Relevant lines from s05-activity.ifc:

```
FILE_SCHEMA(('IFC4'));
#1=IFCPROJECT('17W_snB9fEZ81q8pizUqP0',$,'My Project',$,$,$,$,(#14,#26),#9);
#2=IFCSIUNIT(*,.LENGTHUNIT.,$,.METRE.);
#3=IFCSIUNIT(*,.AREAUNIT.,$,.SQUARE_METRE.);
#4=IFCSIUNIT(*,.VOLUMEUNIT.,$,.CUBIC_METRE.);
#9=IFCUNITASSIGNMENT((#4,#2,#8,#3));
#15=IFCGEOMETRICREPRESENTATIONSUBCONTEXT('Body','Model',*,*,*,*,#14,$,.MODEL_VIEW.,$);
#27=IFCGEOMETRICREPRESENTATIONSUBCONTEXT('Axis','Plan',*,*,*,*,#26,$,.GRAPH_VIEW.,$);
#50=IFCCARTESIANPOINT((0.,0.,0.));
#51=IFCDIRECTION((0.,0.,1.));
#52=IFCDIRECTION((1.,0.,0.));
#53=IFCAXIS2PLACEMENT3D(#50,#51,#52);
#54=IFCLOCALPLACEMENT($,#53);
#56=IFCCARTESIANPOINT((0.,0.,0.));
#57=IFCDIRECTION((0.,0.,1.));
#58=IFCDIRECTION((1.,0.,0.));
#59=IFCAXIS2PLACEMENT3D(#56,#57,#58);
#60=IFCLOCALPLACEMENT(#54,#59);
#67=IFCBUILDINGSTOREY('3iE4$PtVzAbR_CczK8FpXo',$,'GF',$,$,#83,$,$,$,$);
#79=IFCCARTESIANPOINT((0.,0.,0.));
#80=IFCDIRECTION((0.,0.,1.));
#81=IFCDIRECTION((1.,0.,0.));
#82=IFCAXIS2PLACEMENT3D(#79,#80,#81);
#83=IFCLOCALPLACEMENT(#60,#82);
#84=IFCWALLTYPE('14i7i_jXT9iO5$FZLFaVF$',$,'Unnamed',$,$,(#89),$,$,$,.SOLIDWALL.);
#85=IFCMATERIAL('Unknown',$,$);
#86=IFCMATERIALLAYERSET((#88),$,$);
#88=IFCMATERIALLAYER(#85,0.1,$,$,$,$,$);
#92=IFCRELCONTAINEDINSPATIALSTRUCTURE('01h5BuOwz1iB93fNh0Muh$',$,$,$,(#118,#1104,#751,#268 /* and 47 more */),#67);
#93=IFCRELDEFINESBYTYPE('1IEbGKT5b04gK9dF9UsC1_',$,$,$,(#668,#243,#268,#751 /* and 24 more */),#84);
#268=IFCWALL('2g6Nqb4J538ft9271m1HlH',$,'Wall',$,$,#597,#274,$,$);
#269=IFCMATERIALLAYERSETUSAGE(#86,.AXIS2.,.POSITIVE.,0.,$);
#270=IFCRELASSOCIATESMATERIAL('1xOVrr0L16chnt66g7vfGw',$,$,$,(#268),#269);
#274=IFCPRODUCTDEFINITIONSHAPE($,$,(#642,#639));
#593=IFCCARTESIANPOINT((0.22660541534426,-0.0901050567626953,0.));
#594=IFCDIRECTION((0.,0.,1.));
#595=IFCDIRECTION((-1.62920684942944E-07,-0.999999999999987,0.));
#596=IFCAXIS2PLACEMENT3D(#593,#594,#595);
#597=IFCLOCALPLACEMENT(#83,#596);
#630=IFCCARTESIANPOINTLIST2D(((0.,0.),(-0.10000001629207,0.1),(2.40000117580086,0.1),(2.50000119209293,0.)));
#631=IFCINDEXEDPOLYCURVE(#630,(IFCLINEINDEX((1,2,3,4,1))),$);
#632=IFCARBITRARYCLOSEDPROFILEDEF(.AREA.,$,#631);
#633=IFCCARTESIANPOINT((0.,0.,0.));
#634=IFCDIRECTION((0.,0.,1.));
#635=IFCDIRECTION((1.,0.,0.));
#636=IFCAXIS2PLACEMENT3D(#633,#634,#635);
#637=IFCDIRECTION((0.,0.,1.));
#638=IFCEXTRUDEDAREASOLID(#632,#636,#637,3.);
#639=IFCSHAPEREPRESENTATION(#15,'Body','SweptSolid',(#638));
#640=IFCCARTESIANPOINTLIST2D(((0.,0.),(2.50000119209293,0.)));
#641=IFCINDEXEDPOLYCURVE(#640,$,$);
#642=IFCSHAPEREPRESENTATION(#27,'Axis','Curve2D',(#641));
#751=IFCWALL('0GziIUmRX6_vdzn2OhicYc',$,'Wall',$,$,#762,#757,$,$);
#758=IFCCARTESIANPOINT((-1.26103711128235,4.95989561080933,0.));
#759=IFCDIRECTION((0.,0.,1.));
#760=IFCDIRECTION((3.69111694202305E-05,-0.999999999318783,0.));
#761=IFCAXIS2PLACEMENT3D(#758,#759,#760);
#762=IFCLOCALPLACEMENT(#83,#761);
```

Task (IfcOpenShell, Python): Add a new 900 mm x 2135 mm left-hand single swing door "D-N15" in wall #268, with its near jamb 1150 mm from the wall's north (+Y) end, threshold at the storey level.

```python
import numpy as np
import ifcopenshell
import ifcopenshell.api.feature
import ifcopenshell.api.geometry
import ifcopenshell.api.root
import ifcopenshell.api.spatial
import ifcopenshell.geom
import ifcopenshell.util.element
import ifcopenshell.util.placement
import ifcopenshell.util.representation
import ifcopenshell.util.shape
import ifcopenshell.util.unit

model = ifcopenshell.open("s05-activity.ifc")
unit_scale = ifcopenshell.util.unit.calculate_unit_scale(model)
settings = ifcopenshell.geom.settings()


def volume(element):
    """Net volume in cubic metres, openings subtracted."""
    shape = ifcopenshell.geom.create_shape(settings, element)
    return ifcopenshell.util.shape.get_volume(shape.geometry)


wall = model.by_guid("2g6Nqb4J538ft9271m1HlH")
storey = ifcopenshell.util.element.get_container(wall, ifc_class="IfcBuildingStorey")
context = ifcopenshell.util.representation.get_context(model, "Model", "Body", "MODEL_VIEW")
before = volume(wall)

width, height, from_end, sill = 0.9, 2.135, 1.15, 0.0  # metres

# The wall runs along its own X axis, and the end named is its -X end.
wall_shape = ifcopenshell.geom.create_shape(settings, wall)
x, y, z = ifcopenshell.util.shape.get_vertices(wall_shape.geometry).T
start = x.min() + from_end
face, thickness = float(y.min()), float(y.max() - y.min())
wall_matrix = ifcopenshell.util.placement.get_local_placement(wall.ObjectPlacement)
level = ifcopenshell.util.placement.get_local_placement(storey.ObjectPlacement)[2, 3]


def in_wall(x, y):
    """Placement at x, y metres in the wall's axes, at sill height."""
    matrix = wall_matrix.copy()
    matrix[:, 3] = wall_matrix @ np.array([x / unit_scale, y / unit_scale, 0.0, 1.0])
    matrix[2, 3] = level + sill / unit_scale
    return matrix


# Opening: a box that overshoots both wall faces by 50 mm.
opening = ifcopenshell.api.root.create_entity(model, ifc_class="IfcOpeningElement", predefined_type="OPENING")
box = ifcopenshell.api.geometry.add_wall_representation(
    model, context=context, length=width, height=height, thickness=thickness + 0.1
)
ifcopenshell.api.geometry.assign_representation(model, product=opening, representation=box)
ifcopenshell.api.geometry.edit_object_placement(model, product=opening, matrix=in_wall(start, face - 0.05), is_si=False)
ifcopenshell.api.feature.add_feature(model, feature=opening, element=wall)

door = ifcopenshell.api.root.create_entity(model, ifc_class="IfcDoor", name="D-N15", predefined_type="DOOR")
door.OverallWidth, door.OverallHeight = width / unit_scale, height / unit_scale
door.OperationType = "SINGLE_SWING_LEFT"
body = ifcopenshell.api.geometry.add_door_representation(
    model,
    context=context,
    overall_width=door.OverallWidth,
    overall_height=door.OverallHeight,
    operation_type="SINGLE_SWING_LEFT",
    lining_properties={"LiningDepth": thickness / unit_scale, "ThresholdDepth": thickness / unit_scale},
)
ifcopenshell.api.geometry.assign_representation(model, product=door, representation=body)
ifcopenshell.api.spatial.assign_container(model, products=[door], relating_structure=storey)
ifcopenshell.api.feature.add_filling(model, opening=opening, element=door)

# The lining spans the wall, so the door starts at the wall face.
ifcopenshell.api.geometry.edit_object_placement(model, product=door, matrix=in_wall(start, face), is_si=False)

after = volume(wall)

print(f"wall volume {before:.3f} -> {after:.3f} m3")

model.write("s05-activity_rev.ifc")
```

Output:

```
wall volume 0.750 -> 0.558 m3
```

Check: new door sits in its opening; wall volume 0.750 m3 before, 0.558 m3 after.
